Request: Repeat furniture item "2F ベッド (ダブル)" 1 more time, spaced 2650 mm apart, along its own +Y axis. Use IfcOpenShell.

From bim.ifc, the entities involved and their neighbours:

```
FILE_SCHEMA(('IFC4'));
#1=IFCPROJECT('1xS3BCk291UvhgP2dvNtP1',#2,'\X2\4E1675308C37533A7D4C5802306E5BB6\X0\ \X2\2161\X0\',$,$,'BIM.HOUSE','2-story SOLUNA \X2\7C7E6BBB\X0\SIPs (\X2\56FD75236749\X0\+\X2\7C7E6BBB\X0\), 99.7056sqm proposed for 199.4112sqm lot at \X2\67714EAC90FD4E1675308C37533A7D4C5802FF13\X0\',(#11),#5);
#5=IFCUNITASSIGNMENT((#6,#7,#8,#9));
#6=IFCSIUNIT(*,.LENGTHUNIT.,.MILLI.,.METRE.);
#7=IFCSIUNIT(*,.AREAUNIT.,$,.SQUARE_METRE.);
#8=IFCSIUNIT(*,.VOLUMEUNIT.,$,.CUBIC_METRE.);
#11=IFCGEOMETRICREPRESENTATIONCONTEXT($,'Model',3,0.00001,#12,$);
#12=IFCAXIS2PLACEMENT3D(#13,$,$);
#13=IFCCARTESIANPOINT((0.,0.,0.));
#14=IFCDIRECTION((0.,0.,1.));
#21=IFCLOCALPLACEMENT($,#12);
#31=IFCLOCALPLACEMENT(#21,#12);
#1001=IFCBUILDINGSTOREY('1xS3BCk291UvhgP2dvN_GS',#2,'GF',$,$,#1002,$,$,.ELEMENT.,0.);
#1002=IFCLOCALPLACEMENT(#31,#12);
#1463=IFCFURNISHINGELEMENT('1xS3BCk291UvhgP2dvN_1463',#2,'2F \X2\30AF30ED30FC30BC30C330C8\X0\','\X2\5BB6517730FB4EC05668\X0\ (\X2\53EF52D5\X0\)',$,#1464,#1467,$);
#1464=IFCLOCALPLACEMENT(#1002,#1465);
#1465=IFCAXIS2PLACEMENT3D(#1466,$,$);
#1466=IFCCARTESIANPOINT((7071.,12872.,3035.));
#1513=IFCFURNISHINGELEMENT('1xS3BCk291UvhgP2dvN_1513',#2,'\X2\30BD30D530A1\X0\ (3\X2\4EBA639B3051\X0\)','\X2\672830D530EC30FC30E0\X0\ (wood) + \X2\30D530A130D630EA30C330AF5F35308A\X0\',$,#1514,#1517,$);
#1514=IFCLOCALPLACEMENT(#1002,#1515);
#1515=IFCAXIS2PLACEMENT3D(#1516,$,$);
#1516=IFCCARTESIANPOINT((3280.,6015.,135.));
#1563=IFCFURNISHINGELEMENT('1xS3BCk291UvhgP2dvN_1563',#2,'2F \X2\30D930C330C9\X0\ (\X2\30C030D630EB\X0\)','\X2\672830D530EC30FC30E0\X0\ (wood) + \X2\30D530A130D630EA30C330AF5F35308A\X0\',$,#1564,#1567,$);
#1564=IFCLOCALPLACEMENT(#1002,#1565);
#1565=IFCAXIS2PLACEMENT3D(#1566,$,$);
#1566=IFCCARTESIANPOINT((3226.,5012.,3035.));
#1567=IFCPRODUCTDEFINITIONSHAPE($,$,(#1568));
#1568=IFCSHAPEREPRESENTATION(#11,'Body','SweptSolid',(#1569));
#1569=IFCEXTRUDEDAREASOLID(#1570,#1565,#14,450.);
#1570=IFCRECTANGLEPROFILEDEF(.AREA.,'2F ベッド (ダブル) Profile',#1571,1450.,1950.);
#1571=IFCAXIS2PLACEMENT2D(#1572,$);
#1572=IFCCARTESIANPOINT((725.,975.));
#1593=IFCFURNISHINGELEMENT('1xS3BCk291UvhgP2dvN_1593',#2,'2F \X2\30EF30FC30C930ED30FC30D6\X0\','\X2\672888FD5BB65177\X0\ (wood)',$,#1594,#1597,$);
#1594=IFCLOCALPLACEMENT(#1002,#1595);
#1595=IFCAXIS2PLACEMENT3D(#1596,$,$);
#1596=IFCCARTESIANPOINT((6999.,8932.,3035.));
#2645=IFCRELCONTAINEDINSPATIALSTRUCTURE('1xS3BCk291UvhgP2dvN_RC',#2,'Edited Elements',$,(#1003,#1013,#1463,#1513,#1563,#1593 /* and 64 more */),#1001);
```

```python
import ifcopenshell
import ifcopenshell.api.geometry
import ifcopenshell.api.root
import ifcopenshell.util.element
import ifcopenshell.util.placement

model = ifcopenshell.open("bim.ifc")


def reuse_history(source, copy):
    """copy_class also copies each property set's owner history, people and application; keep the originals."""
    for rel in copy.IsDefinedBy:
        if rel.is_a("IfcRelDefinesByProperties") and (history := rel.RelatingPropertyDefinition.OwnerHistory):
            rel.RelatingPropertyDefinition.OwnerHistory = source.OwnerHistory
            ifcopenshell.util.element.remove_deep2(model, history)


source = model.by_guid("1xS3BCk291UvhgP2dvN_1563")
base = ifcopenshell.util.placement.get_local_placement(source.ObjectPlacement)
step = base[:3, 1] * 2650.0

for i in range(1, 2):
    copy = ifcopenshell.api.root.copy_class(model, product=source)
    copy.Representation = ifcopenshell.util.element.copy_deep(
        model, source.Representation, exclude=["IfcGeometricRepresentationContext", "IfcRepresentationMap"]
    )
    reuse_history(source, copy)
    matrix = base.copy()
    matrix[:3, 3] += i * step
    print("added at", matrix[:3, 3].round(3) + 0.0)
    ifcopenshell.api.geometry.edit_object_placement(model, product=copy, matrix=matrix, is_si=False)

model.write("bim_rev.ifc")
```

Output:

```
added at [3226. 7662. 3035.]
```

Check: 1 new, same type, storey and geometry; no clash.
